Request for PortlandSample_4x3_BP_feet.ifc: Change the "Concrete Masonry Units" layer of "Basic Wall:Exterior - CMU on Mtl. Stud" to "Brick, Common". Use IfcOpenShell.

First a look at what the model holds.

```python
import ifcopenshell
import ifcopenshell.util.element

model = ifcopenshell.open("PortlandSample_4x3_BP_feet.ifc")
print(model.schema)
for layer_set in model.by_type("IfcMaterialLayerSet"):
    if layer_set.LayerSetName == "Basic Wall:Exterior - CMU on Mtl. Stud":
        for layer in layer_set.MaterialLayers:
            print(layer.id(), layer.Material and layer.Material.Name, layer.LayerThickness, sep=" | ")
        print(len(ifcopenshell.util.element.get_elements_by_material(model, layer_set)), "elements and types use it")
print(sorted(m.Name for m in model.by_type("IfcMaterial") if m.Name)[:60])
```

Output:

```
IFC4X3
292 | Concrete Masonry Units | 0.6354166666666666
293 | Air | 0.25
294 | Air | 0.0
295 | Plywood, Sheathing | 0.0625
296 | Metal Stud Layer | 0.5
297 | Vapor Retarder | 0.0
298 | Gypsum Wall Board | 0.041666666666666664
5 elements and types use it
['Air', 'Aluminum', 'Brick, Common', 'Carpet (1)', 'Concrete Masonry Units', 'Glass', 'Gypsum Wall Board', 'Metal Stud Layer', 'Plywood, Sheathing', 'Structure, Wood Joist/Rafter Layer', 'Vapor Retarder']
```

```python
import ifcopenshell
import ifcopenshell.api.material

model = ifcopenshell.open("PortlandSample_4x3_BP_feet.ifc")

layer_set = next(s for s in model.by_type("IfcMaterialLayerSet") if s.LayerSetName == "Basic Wall:Exterior - CMU on Mtl. Stud")
layer = next(l for l in layer_set.MaterialLayers if l.Material and l.Material.Name == "Concrete Masonry Units")
material = next(m for m in model.by_type("IfcMaterial") if m.Name == "Brick, Common")

# Point this one layer at the other material; renaming the old one would change it everywhere.
ifcopenshell.api.material.edit_layer(model, layer=layer, attributes={"Name": material.Name}, material=material)

print([l.Material.Name if l.Material else None for l in layer_set.MaterialLayers])

model.write("PortlandSample_4x3_BP_feet_rev.ifc")
```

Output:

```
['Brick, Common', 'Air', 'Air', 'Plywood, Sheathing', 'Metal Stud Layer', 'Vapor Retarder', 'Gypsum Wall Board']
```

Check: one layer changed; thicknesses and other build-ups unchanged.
